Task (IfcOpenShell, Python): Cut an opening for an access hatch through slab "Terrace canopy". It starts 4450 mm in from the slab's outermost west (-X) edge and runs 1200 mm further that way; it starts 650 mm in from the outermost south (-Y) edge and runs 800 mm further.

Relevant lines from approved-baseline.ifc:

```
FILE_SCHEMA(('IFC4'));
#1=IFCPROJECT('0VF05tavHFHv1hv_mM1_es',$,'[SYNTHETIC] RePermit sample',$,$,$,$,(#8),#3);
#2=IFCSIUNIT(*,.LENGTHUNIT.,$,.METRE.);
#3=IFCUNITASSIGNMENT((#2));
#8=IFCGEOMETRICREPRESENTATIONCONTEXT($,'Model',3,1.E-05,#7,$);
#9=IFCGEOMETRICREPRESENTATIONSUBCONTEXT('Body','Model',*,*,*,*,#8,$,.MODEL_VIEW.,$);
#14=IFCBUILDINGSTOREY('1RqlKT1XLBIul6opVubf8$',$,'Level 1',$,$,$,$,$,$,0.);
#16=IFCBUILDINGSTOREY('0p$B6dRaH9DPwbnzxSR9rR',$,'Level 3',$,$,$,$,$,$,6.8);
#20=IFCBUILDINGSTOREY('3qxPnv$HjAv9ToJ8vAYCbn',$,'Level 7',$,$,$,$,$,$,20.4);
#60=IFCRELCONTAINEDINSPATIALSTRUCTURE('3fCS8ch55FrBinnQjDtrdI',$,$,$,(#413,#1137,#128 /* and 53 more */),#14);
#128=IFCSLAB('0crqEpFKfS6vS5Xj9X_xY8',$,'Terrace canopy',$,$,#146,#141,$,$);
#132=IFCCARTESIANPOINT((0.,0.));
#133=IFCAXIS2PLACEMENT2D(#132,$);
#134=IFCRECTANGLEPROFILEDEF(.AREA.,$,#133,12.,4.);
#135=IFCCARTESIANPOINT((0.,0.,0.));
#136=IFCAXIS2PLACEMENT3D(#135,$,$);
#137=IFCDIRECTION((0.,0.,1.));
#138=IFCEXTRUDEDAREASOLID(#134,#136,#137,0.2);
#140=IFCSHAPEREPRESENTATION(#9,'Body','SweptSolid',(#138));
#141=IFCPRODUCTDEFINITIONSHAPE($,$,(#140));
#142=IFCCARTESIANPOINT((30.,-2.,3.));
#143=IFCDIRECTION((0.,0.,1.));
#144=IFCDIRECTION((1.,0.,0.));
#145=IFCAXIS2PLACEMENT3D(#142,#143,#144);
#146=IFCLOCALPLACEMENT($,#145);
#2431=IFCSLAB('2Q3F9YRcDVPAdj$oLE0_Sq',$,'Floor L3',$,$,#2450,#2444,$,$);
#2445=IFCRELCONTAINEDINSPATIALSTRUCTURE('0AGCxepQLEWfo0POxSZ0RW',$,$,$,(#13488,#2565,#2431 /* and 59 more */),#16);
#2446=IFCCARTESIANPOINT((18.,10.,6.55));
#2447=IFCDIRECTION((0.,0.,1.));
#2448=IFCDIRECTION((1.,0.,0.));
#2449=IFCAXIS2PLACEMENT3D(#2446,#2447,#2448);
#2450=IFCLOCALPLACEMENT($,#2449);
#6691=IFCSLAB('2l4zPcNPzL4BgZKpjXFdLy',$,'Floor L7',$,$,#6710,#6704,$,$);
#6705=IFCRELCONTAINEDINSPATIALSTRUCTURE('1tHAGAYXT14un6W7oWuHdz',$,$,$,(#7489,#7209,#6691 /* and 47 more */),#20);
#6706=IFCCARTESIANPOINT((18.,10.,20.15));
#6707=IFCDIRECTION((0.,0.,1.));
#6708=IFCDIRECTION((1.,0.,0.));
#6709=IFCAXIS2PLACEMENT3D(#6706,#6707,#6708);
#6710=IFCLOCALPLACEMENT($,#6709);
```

```python
import numpy as np
import ifcopenshell
import ifcopenshell.api.feature
import ifcopenshell.api.geometry
import ifcopenshell.api.root
import ifcopenshell.geom
import ifcopenshell.util.placement
import ifcopenshell.util.representation
import ifcopenshell.util.shape
import ifcopenshell.util.unit

model = ifcopenshell.open("approved-baseline.ifc")
unit_scale = ifcopenshell.util.unit.calculate_unit_scale(model)
settings = ifcopenshell.geom.settings()


def volume(element):
    """Net volume in cubic metres, openings subtracted."""
    shape = ifcopenshell.geom.create_shape(settings, element)
    return ifcopenshell.util.shape.get_volume(shape.geometry)


slab = model.by_guid("0crqEpFKfS6vS5Xj9X_xY8")
before = volume(slab)

# Extent in the slab's own axes, in metres. The edges named are its -X and -Y sides.
slab_shape = ifcopenshell.geom.create_shape(settings, slab)
vertices = ifcopenshell.util.shape.get_vertices(slab_shape.geometry)
x_min, y_min, bottom = vertices.min(axis=0)
top = vertices[:, 2].max()

opening = ifcopenshell.api.root.create_entity(model, ifc_class="IfcOpeningElement", name="Access hatch opening", predefined_type="OPENING")
context = ifcopenshell.util.representation.get_context(model, "Model", "Body", "MODEL_VIEW")
width, depth = 1.2, 0.8
outline = [(0.0, 0.0), (width, 0.0), (width, depth), (0.0, depth), (0.0, 0.0)]
# Overshoot both faces by 50 mm so the cut is clean.
shape = ifcopenshell.api.geometry.add_slab_representation(
    model, context=context, depth=top - bottom + 0.1, polyline=outline
)
ifcopenshell.api.geometry.assign_representation(model, product=opening, representation=shape)

matrix = ifcopenshell.util.placement.get_local_placement(slab.ObjectPlacement)
matrix[:, 3] = matrix @ np.append(np.array([x_min + 4.45, y_min + 0.65, bottom - 0.05]) / unit_scale, 1.0)
ifcopenshell.api.geometry.edit_object_placement(model, product=opening, matrix=matrix, is_si=False)
ifcopenshell.api.feature.add_feature(model, feature=opening, element=slab)

after = volume(slab)

print(f"slab volume {before:.3f} -> {after:.3f} m3")

model.write("approved-baseline-out.ifc")
```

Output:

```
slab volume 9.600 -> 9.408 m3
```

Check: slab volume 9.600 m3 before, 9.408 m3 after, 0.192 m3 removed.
